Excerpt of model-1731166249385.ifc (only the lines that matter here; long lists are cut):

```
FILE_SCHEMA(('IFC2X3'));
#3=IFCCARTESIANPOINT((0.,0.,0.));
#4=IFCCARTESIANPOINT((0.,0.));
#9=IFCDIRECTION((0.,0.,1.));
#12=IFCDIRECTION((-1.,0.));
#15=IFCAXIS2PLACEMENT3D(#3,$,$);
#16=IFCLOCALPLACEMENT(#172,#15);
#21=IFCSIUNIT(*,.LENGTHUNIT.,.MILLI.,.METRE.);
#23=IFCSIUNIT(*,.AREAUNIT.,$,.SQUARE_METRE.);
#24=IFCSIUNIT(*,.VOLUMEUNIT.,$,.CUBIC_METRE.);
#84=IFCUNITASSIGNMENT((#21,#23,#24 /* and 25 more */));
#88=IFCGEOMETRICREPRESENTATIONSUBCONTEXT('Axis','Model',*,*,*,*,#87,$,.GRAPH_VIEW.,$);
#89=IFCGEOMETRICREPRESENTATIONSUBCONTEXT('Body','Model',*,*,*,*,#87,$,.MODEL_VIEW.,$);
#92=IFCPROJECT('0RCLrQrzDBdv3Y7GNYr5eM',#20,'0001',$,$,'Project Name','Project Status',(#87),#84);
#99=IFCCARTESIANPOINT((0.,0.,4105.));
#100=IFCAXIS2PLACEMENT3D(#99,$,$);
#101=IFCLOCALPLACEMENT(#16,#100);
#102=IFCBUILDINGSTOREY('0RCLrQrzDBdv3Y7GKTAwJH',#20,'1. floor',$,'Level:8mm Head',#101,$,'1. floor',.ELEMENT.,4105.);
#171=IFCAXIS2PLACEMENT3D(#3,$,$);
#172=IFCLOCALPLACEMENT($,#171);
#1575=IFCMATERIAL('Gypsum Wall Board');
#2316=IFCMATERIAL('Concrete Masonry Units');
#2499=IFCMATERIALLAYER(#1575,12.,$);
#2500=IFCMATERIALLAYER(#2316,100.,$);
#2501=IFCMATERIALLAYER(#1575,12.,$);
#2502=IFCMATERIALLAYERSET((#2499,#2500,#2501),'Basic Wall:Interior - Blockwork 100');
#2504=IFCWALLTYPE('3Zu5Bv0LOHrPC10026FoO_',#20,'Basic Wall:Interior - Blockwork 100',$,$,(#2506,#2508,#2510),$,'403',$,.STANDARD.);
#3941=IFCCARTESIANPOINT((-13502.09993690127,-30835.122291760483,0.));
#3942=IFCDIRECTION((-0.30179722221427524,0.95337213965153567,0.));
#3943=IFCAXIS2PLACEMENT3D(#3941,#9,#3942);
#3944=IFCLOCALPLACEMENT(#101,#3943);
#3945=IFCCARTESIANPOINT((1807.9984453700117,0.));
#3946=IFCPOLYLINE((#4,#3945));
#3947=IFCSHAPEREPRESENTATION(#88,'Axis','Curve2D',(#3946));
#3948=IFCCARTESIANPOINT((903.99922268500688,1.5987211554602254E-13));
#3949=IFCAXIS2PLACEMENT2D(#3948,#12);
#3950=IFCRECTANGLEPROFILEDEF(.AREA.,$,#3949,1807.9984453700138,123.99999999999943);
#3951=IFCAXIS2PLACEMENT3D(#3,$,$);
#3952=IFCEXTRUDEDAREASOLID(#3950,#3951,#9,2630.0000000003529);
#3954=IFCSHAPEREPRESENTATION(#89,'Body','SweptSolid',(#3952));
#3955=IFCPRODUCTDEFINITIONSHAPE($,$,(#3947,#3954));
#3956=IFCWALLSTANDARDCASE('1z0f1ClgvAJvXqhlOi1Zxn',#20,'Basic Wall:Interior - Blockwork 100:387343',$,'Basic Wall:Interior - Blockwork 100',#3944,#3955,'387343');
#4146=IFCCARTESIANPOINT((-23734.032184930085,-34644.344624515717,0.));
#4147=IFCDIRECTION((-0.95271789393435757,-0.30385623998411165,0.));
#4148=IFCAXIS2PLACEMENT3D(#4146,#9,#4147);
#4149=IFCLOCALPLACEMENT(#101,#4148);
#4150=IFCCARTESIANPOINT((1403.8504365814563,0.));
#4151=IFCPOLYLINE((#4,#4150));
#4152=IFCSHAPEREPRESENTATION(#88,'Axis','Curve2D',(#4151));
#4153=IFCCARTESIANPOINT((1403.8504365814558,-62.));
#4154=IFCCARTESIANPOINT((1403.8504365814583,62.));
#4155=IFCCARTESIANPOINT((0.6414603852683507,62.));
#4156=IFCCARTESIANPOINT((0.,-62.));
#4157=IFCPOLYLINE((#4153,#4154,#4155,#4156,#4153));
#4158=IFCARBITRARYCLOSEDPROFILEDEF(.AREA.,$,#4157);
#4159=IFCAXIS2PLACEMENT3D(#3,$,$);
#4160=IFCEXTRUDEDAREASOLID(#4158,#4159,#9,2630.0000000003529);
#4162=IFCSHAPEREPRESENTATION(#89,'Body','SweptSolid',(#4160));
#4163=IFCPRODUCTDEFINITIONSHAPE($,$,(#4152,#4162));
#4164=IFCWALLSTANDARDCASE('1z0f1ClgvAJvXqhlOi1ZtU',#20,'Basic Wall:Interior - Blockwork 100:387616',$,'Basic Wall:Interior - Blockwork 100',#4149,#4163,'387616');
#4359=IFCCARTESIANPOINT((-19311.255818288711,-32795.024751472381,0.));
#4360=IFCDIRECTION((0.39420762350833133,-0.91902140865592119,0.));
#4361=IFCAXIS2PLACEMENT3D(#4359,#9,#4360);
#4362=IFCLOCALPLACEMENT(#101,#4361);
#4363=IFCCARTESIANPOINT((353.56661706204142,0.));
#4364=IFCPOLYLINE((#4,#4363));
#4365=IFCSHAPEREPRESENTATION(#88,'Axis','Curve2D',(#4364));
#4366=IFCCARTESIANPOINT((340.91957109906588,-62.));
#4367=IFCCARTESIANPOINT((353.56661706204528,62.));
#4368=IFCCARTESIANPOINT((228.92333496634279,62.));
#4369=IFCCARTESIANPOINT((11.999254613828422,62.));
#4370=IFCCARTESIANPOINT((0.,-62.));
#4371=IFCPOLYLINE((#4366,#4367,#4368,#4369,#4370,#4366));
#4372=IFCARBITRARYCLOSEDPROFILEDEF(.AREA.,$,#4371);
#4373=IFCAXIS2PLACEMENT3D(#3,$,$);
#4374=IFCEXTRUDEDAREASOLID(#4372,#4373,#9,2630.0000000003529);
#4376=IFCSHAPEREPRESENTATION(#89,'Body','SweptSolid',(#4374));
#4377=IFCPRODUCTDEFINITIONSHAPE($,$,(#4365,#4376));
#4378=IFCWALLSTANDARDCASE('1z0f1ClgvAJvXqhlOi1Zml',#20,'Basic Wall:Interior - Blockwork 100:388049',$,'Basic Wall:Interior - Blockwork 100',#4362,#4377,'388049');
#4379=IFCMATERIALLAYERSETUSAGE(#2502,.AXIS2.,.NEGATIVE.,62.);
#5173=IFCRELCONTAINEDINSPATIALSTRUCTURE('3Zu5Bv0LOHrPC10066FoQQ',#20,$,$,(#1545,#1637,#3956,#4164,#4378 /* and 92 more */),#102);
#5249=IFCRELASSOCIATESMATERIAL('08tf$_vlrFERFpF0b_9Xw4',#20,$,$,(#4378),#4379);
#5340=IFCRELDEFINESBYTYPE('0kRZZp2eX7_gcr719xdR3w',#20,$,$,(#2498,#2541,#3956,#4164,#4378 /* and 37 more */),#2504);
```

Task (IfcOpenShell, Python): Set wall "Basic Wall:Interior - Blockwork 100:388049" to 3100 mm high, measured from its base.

```python
import ifcopenshell
import ifcopenshell.geom
import ifcopenshell.util.representation
import ifcopenshell.util.shape

model = ifcopenshell.open("model-1731166249385.ifc")
settings = ifcopenshell.geom.settings()


def volume(element):
    """Net volume in cubic metres, openings subtracted."""
    shape = ifcopenshell.geom.create_shape(settings, element)
    return ifcopenshell.util.shape.get_volume(shape.geometry)


wall = model.by_id(4378)
before = volume(wall)

body = ifcopenshell.util.representation.get_representation(wall, "Model", "Body")
solid = body.Items[0]
old_height = solid.Depth
solid.Depth = 3100.0
after = volume(wall)

print(f"height {old_height:g} -> {solid.Depth:g}, volume {before:.3f} -> {after:.3f} m3")

model.write("model-1731166249385_rev.ifc")
```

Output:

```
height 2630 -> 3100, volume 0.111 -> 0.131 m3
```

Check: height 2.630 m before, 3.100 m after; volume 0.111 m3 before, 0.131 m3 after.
